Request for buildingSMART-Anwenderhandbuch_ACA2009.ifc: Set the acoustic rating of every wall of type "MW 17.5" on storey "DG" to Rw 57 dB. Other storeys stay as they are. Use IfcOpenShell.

First a look at what the model holds.

```python
import ifcopenshell
import ifcopenshell.util.element

model = ifcopenshell.open("buildingSMART-Anwenderhandbuch_ACA2009.ifc")
print(model.schema)
storey = next(s for s in model.by_type("IfcBuildingStorey") if s.Name == "DG")
walls = [e for e in ifcopenshell.util.element.get_decomposition(storey) if e.is_a("IfcWall")]
seen = {}
for e in walls:
    element_type = ifcopenshell.util.element.get_type(e)
    key = (element_type.Name if element_type != e and element_type else None, ifcopenshell.util.element.get_pset(e, "Pset_WallCommon", "AcousticRating"))
    seen[key] = seen.get(key, 0) + 1
for (name, value), count in sorted(seen.items(), key=str):
    print(count, "x", name, "|", value)
```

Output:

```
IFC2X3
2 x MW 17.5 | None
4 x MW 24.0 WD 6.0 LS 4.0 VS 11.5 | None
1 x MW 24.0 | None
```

```python
import ifcopenshell
import ifcopenshell.api.pset
import ifcopenshell.util.element

model = ifcopenshell.open("buildingSMART-Anwenderhandbuch_ACA2009.ifc")

storey = next(s for s in model.by_type("IfcBuildingStorey") if s.Name == "DG")
walls = [e for e in ifcopenshell.util.element.get_decomposition(storey) if e.is_a("IfcWall")]

count = 0
for e in walls:
    element_type = ifcopenshell.util.element.get_type(e)
    if element_type in (None, e) or element_type.Name != "MW 17.5":
        continue
    # add_pset returns the element's existing set when there is one.
    pset = ifcopenshell.api.pset.add_pset(model, product=e, name="Pset_WallCommon")
    ifcopenshell.api.pset.edit_pset(model, pset=pset, properties={"AcousticRating": "Rw 57 dB"})
    count += 1

print(count, "walls updated")

model.write("buildingSMART-Anwenderhandbuch_ACA2009_edited.ifc")
```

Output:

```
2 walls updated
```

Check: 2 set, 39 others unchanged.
